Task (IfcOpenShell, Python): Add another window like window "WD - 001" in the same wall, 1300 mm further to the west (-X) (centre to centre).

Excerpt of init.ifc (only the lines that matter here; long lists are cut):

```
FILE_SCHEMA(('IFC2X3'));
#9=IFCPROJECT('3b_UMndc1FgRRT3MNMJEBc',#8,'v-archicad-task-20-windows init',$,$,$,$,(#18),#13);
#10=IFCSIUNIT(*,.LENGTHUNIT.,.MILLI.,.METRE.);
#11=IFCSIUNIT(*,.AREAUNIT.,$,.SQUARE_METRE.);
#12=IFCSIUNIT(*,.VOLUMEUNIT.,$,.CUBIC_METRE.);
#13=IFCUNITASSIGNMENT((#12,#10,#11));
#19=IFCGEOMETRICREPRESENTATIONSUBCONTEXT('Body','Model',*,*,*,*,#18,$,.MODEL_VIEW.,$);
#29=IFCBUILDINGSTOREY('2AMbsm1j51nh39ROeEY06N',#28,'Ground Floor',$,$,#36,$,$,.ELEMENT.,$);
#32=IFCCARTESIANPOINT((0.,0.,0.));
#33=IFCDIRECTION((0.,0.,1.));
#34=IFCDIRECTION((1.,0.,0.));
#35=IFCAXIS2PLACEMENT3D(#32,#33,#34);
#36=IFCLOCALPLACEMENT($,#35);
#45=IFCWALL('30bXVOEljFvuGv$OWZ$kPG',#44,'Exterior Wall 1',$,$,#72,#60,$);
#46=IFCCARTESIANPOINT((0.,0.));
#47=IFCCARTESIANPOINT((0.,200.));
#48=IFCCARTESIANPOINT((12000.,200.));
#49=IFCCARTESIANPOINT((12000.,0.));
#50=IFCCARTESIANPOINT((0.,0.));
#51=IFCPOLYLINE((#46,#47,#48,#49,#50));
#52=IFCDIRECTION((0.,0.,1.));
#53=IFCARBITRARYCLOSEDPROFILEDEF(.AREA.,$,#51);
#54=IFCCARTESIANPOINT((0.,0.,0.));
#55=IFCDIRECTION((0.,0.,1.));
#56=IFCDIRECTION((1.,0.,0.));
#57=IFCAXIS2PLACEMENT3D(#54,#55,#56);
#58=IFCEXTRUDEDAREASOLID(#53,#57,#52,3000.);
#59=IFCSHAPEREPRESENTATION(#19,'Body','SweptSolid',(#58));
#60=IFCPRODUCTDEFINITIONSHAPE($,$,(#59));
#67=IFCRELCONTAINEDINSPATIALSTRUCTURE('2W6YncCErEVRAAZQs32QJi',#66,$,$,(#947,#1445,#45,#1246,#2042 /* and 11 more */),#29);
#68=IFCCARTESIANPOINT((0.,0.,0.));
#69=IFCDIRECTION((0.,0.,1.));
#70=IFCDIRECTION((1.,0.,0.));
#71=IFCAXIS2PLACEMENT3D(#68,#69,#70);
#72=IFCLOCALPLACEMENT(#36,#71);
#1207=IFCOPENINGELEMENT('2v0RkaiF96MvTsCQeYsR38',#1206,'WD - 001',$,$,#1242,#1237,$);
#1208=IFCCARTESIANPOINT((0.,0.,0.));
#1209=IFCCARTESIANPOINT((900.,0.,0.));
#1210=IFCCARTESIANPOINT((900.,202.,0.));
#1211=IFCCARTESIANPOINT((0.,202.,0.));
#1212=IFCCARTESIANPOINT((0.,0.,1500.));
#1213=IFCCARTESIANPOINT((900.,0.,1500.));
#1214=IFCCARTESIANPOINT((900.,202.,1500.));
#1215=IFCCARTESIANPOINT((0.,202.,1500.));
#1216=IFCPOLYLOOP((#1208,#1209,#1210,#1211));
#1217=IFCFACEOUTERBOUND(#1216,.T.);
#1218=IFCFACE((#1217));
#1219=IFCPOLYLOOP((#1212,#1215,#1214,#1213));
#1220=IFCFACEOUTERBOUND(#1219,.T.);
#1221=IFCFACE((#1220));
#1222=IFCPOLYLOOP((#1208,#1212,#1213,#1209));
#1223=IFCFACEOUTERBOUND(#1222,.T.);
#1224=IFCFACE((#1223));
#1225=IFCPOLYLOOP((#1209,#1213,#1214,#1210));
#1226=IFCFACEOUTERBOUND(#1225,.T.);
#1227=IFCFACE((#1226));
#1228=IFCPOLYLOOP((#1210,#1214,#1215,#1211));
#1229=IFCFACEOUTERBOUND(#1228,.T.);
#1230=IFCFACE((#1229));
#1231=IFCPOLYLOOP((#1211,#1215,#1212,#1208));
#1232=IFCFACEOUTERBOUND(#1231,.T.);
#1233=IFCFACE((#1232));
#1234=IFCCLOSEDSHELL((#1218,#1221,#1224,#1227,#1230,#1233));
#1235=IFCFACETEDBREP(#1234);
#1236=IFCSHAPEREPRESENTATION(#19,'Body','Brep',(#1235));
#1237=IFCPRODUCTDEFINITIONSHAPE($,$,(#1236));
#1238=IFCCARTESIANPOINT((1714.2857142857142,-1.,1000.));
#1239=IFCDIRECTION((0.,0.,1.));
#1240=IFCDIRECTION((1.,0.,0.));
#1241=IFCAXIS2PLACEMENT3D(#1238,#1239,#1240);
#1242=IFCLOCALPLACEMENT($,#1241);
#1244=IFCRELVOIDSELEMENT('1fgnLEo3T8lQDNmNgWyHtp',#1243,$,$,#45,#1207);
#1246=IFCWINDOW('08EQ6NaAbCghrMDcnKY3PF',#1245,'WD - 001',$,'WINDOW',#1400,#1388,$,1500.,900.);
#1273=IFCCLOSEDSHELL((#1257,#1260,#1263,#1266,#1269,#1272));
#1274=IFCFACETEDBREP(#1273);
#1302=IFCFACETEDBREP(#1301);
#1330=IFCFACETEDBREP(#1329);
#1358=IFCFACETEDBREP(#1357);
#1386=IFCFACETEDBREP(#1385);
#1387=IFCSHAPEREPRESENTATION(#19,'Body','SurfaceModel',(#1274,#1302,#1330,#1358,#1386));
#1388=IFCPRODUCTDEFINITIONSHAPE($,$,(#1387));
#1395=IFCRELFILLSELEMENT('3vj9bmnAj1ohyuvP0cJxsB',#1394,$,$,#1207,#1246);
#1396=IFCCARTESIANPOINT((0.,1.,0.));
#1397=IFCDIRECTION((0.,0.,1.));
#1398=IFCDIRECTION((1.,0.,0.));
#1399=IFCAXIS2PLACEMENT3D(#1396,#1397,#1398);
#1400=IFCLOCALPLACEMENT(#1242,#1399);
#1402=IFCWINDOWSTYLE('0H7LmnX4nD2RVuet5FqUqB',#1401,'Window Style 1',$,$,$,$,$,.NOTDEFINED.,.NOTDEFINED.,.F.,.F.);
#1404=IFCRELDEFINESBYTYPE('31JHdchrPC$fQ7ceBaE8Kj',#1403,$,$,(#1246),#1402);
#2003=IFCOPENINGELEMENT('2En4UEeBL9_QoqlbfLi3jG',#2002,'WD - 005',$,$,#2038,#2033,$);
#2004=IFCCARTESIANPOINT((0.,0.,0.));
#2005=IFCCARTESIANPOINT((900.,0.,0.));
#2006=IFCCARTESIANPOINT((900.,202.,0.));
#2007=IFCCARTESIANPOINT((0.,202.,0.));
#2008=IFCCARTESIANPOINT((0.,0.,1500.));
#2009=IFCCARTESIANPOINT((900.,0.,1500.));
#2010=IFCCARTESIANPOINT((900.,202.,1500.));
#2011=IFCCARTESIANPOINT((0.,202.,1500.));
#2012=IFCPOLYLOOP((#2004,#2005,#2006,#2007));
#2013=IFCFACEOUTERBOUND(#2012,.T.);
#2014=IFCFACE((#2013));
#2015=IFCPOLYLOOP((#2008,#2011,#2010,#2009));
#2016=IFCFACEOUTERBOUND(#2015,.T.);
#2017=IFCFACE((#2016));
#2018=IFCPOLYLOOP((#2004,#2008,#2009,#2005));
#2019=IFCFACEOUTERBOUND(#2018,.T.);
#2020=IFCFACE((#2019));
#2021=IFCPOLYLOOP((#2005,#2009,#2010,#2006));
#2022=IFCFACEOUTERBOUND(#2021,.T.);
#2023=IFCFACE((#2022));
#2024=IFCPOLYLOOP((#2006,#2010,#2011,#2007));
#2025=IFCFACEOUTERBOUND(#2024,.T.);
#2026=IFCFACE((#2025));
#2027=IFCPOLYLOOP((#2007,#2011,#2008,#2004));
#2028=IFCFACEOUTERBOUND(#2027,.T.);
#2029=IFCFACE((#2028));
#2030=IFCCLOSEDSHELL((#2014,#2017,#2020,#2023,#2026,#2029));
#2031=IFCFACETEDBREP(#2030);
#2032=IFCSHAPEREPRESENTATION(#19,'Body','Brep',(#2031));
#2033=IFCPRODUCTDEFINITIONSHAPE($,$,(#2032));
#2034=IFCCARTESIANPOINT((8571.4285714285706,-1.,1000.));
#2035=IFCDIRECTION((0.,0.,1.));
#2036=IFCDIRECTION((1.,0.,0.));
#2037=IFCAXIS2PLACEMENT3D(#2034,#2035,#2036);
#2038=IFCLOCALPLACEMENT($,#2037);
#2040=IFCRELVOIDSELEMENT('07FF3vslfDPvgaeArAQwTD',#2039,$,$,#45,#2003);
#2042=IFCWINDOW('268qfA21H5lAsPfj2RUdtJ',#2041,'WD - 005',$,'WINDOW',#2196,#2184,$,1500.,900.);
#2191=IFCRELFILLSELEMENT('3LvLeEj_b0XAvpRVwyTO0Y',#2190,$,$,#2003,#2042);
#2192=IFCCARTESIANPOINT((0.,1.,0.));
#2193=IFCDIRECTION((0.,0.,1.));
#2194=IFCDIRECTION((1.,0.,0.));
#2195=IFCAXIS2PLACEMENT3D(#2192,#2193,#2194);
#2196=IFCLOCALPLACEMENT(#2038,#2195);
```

```python
import ifcopenshell
import ifcopenshell.api.feature
import ifcopenshell.api.geometry
import ifcopenshell.api.root
import ifcopenshell.geom
import ifcopenshell.util.element
import ifcopenshell.util.placement
import ifcopenshell.util.shape
import ifcopenshell.util.unit

model = ifcopenshell.open("init.ifc")
unit_scale = ifcopenshell.util.unit.calculate_unit_scale(model)
settings = ifcopenshell.geom.settings()


def volume(element):
    """Net volume in cubic metres, openings subtracted."""
    shape = ifcopenshell.geom.create_shape(settings, element)
    return ifcopenshell.util.shape.get_volume(shape.geometry)


window = model.by_guid("08EQ6NaAbCghrMDcnKY3PF")
opening = window.FillsVoids[0].RelatingOpeningElement
wall = opening.VoidsElements[0].RelatingBuildingElement
before = volume(wall)
shift = ifcopenshell.util.placement.get_local_placement(wall.ObjectPlacement)[:3, 0] * -1.3 / unit_scale

# copy_class copies the void relationship, type, container and properties, but no geometry.
new_opening = ifcopenshell.api.root.copy_class(model, product=opening)
new_opening.Representation = ifcopenshell.util.element.copy_deep(
    model, opening.Representation, exclude=["IfcGeometricRepresentationContext", "IfcRepresentationMap"]
)
new_window = ifcopenshell.api.root.copy_class(model, product=window)
new_window.Representation = ifcopenshell.util.element.copy_deep(
    model, window.Representation, exclude=["IfcGeometricRepresentationContext", "IfcRepresentationMap"]
)
fills = ifcopenshell.api.feature.add_filling(model, opening=new_opening, element=new_window)
fills.OwnerHistory = new_window.OwnerHistory  # required in IFC2X3

for old, new in ((opening, new_opening), (window, new_window)):
    matrix = ifcopenshell.util.placement.get_local_placement(old.ObjectPlacement)
    matrix[:3, 3] += shift
    ifcopenshell.api.geometry.edit_object_placement(model, product=new, matrix=matrix, is_si=False)

after = volume(wall)

print(f"wall volume {before:.3f} -> {after:.3f} m3")

model.write("init_updated.ifc")
```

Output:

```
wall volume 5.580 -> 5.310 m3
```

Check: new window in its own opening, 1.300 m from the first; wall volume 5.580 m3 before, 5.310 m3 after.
